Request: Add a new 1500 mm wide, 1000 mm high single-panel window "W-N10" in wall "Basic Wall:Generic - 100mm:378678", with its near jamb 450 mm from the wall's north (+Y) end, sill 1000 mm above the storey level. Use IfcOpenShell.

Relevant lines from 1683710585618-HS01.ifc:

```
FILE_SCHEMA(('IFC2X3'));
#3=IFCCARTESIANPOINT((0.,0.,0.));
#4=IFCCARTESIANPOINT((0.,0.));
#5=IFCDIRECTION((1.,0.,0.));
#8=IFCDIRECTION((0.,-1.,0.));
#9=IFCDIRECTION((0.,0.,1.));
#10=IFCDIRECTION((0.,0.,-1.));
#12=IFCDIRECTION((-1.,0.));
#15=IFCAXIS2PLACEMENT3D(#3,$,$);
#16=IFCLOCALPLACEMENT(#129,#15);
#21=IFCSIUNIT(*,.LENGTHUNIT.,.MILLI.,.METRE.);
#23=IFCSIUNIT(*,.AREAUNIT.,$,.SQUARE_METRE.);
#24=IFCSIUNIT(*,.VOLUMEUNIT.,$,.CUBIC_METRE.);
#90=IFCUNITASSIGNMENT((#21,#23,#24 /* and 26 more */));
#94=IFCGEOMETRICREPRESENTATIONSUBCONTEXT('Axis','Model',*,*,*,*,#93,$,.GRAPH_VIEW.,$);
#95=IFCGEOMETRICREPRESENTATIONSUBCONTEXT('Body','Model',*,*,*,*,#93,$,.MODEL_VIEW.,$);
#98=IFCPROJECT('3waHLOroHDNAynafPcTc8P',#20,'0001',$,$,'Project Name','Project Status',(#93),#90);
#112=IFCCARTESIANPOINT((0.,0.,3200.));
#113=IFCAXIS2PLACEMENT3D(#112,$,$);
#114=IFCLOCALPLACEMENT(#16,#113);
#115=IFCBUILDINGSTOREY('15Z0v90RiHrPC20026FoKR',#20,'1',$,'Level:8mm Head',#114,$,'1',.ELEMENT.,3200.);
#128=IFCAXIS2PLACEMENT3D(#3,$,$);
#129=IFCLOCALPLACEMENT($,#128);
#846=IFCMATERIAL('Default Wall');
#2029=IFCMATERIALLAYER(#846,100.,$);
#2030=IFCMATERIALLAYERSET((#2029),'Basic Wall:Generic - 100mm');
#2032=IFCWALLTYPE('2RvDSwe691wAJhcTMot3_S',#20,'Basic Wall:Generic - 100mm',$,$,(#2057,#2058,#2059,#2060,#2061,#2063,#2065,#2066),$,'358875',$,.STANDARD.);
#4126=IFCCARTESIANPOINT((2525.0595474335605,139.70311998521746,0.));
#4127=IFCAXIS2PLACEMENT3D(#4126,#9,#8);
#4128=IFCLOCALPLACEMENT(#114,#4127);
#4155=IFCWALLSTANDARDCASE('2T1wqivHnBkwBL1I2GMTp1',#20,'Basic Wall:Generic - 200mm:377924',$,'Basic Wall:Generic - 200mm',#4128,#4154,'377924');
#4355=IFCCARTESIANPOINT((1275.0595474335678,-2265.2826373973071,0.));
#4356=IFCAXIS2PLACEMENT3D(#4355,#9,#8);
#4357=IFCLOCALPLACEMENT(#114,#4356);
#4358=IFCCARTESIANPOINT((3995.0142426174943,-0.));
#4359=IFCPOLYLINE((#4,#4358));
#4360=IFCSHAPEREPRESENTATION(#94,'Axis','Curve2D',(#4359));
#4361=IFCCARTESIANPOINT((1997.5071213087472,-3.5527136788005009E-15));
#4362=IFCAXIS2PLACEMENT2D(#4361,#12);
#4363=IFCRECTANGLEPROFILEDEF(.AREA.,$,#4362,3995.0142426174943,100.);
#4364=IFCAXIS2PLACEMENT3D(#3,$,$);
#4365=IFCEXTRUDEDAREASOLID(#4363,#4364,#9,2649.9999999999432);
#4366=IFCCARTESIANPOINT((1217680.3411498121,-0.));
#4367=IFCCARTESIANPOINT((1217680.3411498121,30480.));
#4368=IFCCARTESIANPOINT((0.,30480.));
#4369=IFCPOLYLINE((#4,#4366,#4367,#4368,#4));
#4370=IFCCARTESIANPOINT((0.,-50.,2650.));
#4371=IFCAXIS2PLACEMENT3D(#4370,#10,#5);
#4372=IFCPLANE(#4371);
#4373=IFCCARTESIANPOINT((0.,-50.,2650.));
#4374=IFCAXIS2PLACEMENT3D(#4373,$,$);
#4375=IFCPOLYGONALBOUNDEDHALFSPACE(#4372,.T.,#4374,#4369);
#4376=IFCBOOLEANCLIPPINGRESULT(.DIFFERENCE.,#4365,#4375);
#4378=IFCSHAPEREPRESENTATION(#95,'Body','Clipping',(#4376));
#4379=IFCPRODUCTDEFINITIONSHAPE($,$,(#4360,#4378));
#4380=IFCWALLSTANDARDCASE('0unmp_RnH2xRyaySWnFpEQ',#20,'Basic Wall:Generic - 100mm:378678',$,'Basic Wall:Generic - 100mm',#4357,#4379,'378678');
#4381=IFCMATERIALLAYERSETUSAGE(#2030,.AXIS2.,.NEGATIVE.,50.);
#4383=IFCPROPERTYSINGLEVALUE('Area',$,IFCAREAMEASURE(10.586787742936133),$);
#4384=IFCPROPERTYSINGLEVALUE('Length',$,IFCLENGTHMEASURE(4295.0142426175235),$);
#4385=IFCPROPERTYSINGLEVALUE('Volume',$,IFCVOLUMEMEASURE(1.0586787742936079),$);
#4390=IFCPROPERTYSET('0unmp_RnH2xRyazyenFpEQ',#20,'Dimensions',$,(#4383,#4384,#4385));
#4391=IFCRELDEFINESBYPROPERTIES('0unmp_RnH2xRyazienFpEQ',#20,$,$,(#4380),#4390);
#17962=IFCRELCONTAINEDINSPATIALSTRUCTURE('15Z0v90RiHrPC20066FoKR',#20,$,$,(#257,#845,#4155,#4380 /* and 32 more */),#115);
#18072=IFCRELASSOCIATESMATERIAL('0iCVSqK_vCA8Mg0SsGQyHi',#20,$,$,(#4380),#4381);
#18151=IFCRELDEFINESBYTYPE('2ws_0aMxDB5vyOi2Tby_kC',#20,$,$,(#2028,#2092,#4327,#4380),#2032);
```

```python
import numpy as np
import ifcopenshell
import ifcopenshell.api.feature
import ifcopenshell.api.geometry
import ifcopenshell.api.pset
import ifcopenshell.api.root
import ifcopenshell.api.spatial
import ifcopenshell.api.type
import ifcopenshell.geom
import ifcopenshell.util.element
import ifcopenshell.util.placement
import ifcopenshell.util.representation
import ifcopenshell.util.shape
import ifcopenshell.util.unit

model = ifcopenshell.open("1683710585618-HS01.ifc")
unit_scale = ifcopenshell.util.unit.calculate_unit_scale(model)
area_scale = ifcopenshell.util.unit.calculate_unit_scale(model, "AREAUNIT")
volume_scale = ifcopenshell.util.unit.calculate_unit_scale(model, "VOLUMEUNIT")
settings = ifcopenshell.geom.settings()


def volume(element):
    """Net volume in cubic metres, openings subtracted."""
    shape = ifcopenshell.geom.create_shape(settings, element)
    return ifcopenshell.util.shape.get_volume(shape.geometry)


wall = model.by_guid("0unmp_RnH2xRyaySWnFpEQ")
storey = ifcopenshell.util.element.get_container(wall, ifc_class="IfcBuildingStorey")
context = ifcopenshell.util.representation.get_context(model, "Model", "Body", "MODEL_VIEW")
before = volume(wall)

width, height, from_end, sill = 1.5, 1, 0.45, 1  # metres

# The wall runs along its own X axis, and the end named is its -X end.
wall_shape = ifcopenshell.geom.create_shape(settings, wall)
x, y, z = ifcopenshell.util.shape.get_vertices(wall_shape.geometry).T
start = x.min() + from_end
face, thickness = float(y.min()), float(y.max() - y.min())
wall_matrix = ifcopenshell.util.placement.get_local_placement(wall.ObjectPlacement)
level = ifcopenshell.util.placement.get_local_placement(storey.ObjectPlacement)[2, 3]


def in_wall(x, y):
    """Placement at x, y metres in the wall's axes, at sill height."""
    matrix = wall_matrix.copy()
    matrix[:, 3] = wall_matrix @ np.array([x / unit_scale, y / unit_scale, 0.0, 1.0])
    matrix[2, 3] = level + sill / unit_scale
    return matrix


# Opening: a box that overshoots both wall faces by 50 mm.
opening = ifcopenshell.api.root.create_entity(model, ifc_class="IfcOpeningElement")
box = ifcopenshell.api.geometry.add_wall_representation(
    model, context=context, length=width, height=height, thickness=thickness + 0.1
)
ifcopenshell.api.geometry.assign_representation(model, product=opening, representation=box)
ifcopenshell.api.geometry.edit_object_placement(model, product=opening, matrix=in_wall(start, face - 0.05), is_si=False)
ifcopenshell.api.feature.add_feature(model, feature=opening, element=wall)

window = ifcopenshell.api.root.create_entity(model, ifc_class="IfcWindow", name="W-N10")
window.OverallWidth, window.OverallHeight = width / unit_scale, height / unit_scale
body = ifcopenshell.api.geometry.add_window_representation(
    model,
    context=context,
    overall_width=window.OverallWidth,
    overall_height=window.OverallHeight,
    partition_type="SINGLE_PANEL",
)
ifcopenshell.api.geometry.assign_representation(model, product=window, representation=body)
ifcopenshell.api.spatial.assign_container(model, products=[window], relating_structure=storey)
fills = ifcopenshell.api.feature.add_filling(model, opening=opening, element=window)
fills.OwnerHistory = window.OwnerHistory  # required in IFC2X3

# IFC2X3 keeps the operation on the window style.
style = ifcopenshell.api.root.create_entity(model, ifc_class="IfcWindowStyle", name="W-N10")
style.OperationType, style.ConstructionType = "SINGLE_PANEL", "NOTDEFINED"
style.ParameterTakesPrecedence = style.Sizeable = False
ifcopenshell.api.type.assign_type(model, related_objects=[window], relating_type=style)

# Centre the window in the wall's thickness.
ifcopenshell.api.geometry.edit_object_placement(model, product=window, matrix=in_wall(start, face), is_si=False)
window_shape = ifcopenshell.geom.create_shape(settings, window)
depth = ifcopenshell.util.shape.get_vertices(window_shape.geometry)[:, 1]
offset = face + thickness / 2 - (depth.min() + depth.max()) / 2
ifcopenshell.api.geometry.edit_object_placement(model, product=window, matrix=in_wall(start, offset), is_si=False)

after = volume(wall)

# Update the wall's stored quantities.
pset = model.by_id(ifcopenshell.util.element.get_pset(wall, "Dimensions", should_inherit=False)["id"])
ifcopenshell.api.pset.edit_pset(model, pset=pset, properties={
    "Area": model.create_entity("IfcAreaMeasure", after / thickness / area_scale),
    "Volume": model.create_entity("IfcVolumeMeasure", after / volume_scale),
})

print(f"wall volume {before:.3f} -> {after:.3f} m3")

model.write("1683710585618-HS01_edited.ifc")
```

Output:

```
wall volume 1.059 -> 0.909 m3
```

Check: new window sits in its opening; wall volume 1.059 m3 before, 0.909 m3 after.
